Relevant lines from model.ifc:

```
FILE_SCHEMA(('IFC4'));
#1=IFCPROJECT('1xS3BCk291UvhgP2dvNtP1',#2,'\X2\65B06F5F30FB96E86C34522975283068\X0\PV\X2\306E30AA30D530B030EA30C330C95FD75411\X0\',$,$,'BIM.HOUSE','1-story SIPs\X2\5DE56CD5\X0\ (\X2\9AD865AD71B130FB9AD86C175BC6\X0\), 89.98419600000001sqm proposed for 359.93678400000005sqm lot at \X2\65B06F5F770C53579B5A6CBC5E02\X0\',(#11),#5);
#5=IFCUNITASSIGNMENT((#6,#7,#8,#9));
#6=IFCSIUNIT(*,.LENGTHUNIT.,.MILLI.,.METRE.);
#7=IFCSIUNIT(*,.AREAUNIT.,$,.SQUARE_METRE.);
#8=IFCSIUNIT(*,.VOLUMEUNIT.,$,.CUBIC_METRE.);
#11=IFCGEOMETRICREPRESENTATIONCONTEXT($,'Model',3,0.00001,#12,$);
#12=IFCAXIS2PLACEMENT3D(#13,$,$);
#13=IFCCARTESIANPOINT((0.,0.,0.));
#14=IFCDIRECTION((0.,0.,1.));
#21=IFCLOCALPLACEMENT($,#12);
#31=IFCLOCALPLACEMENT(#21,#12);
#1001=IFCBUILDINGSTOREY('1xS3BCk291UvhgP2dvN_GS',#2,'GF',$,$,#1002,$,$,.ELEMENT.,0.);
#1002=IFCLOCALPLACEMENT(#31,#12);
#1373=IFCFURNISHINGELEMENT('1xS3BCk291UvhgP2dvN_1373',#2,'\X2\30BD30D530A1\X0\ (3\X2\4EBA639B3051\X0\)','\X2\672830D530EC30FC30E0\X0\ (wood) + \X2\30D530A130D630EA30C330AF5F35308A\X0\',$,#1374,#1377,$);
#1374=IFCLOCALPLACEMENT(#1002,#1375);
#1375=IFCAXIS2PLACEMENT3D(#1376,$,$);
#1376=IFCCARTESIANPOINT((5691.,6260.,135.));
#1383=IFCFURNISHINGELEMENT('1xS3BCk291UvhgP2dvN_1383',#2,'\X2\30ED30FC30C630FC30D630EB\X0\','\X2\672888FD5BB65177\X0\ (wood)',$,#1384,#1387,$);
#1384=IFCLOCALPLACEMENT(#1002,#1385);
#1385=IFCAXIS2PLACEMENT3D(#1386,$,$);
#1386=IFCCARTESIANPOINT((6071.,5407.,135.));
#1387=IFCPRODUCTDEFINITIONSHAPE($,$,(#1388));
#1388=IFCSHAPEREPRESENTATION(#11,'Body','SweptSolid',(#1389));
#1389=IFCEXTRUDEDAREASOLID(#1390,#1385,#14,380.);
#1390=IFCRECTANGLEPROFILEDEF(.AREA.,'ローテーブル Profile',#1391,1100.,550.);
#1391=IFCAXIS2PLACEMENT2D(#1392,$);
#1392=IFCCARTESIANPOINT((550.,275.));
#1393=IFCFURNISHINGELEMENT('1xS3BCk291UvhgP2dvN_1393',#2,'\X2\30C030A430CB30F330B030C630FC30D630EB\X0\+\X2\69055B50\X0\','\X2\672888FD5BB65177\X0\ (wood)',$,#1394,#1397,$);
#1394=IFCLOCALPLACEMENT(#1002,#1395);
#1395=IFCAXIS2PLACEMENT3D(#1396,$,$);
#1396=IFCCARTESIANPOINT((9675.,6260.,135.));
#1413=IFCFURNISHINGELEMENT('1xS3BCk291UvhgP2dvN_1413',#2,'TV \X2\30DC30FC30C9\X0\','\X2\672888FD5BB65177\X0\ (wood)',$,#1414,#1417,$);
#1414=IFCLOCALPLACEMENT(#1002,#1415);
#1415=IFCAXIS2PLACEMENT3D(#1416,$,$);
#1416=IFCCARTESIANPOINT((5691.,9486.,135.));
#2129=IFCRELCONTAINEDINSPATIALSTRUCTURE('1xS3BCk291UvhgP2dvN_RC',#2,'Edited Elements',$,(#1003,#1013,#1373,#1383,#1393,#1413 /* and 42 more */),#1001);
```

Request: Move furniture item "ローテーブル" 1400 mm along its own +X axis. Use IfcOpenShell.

```python
import ifcopenshell
import ifcopenshell.api.geometry
import ifcopenshell.util.placement
import ifcopenshell.util.unit

model = ifcopenshell.open("model.ifc")
unit_scale = ifcopenshell.util.unit.calculate_unit_scale(model)

item = model.by_id(1383)
matrix = ifcopenshell.util.placement.get_local_placement(item.ObjectPlacement)
matrix[:3, 3] += matrix[:3, 0] * 1.4 / unit_scale
ifcopenshell.api.geometry.edit_object_placement(model, product=item, matrix=matrix, is_si=False)

print(ifcopenshell.util.placement.get_local_placement(item.ObjectPlacement).round(3) + 0.0)

model.write("model_v2.ifc")
```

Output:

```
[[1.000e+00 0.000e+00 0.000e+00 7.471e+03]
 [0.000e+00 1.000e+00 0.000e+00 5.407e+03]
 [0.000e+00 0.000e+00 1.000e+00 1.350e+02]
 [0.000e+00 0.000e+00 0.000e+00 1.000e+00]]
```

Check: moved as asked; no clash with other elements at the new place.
